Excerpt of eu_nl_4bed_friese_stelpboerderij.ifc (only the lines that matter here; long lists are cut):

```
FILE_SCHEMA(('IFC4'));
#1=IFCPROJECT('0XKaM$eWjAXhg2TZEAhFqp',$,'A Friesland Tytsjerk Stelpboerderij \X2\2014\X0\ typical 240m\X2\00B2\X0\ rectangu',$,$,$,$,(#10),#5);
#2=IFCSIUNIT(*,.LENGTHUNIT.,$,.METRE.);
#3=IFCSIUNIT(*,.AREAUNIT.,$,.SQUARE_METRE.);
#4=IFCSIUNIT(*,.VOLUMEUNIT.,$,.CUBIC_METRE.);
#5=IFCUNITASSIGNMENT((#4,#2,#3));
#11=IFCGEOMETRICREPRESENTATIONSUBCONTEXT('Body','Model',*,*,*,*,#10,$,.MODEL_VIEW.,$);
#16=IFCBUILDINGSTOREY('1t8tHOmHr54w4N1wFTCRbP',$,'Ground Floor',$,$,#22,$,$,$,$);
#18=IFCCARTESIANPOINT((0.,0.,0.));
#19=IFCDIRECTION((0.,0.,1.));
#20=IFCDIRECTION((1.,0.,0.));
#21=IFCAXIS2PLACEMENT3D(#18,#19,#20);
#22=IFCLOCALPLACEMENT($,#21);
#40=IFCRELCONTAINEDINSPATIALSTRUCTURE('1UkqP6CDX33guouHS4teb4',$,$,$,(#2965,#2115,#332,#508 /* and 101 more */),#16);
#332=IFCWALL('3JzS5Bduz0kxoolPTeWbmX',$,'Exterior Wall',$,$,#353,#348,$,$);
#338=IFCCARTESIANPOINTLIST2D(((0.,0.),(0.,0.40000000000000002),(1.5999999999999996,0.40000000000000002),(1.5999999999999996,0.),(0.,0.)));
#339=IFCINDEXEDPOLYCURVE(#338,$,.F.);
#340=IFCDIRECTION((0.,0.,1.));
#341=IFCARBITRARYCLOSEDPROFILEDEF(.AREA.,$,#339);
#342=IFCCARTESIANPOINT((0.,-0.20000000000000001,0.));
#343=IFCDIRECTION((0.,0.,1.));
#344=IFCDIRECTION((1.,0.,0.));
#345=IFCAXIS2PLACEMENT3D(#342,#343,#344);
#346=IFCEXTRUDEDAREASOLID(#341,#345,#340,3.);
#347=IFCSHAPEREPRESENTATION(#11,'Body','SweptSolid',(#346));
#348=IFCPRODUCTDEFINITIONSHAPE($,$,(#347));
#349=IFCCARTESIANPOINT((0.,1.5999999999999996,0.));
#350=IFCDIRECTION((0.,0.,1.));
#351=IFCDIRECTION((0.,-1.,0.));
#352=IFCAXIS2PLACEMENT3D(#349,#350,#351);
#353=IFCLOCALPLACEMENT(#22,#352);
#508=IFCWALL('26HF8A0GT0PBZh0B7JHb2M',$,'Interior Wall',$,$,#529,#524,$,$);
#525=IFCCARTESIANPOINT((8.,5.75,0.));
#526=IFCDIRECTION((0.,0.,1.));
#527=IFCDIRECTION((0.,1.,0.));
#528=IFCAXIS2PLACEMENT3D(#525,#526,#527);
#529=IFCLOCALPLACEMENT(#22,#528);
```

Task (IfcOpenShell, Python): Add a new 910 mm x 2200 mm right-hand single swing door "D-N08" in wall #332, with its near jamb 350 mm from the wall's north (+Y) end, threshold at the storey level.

```python
import numpy as np
import ifcopenshell
import ifcopenshell.api.feature
import ifcopenshell.api.geometry
import ifcopenshell.api.root
import ifcopenshell.api.spatial
import ifcopenshell.geom
import ifcopenshell.util.element
import ifcopenshell.util.placement
import ifcopenshell.util.representation
import ifcopenshell.util.shape
import ifcopenshell.util.unit

model = ifcopenshell.open("eu_nl_4bed_friese_stelpboerderij.ifc")
unit_scale = ifcopenshell.util.unit.calculate_unit_scale(model)
settings = ifcopenshell.geom.settings()


def volume(element):
    """Net volume in cubic metres, openings subtracted."""
    shape = ifcopenshell.geom.create_shape(settings, element)
    return ifcopenshell.util.shape.get_volume(shape.geometry)


wall = model.by_id(332)
storey = ifcopenshell.util.element.get_container(wall, ifc_class="IfcBuildingStorey")
context = ifcopenshell.util.representation.get_context(model, "Model", "Body", "MODEL_VIEW")
before = volume(wall)

width, height, from_end, sill = 0.91, 2.2, 0.35, 0.0  # metres

# The wall runs along its own X axis, and the end named is its -X end.
wall_shape = ifcopenshell.geom.create_shape(settings, wall)
x, y, z = ifcopenshell.util.shape.get_vertices(wall_shape.geometry).T
start = x.min() + from_end
face, thickness = float(y.min()), float(y.max() - y.min())
wall_matrix = ifcopenshell.util.placement.get_local_placement(wall.ObjectPlacement)
level = ifcopenshell.util.placement.get_local_placement(storey.ObjectPlacement)[2, 3]


def in_wall(x, y):
    """Placement at x, y metres in the wall's axes, at sill height."""
    matrix = wall_matrix.copy()
    matrix[:, 3] = wall_matrix @ np.array([x / unit_scale, y / unit_scale, 0.0, 1.0])
    matrix[2, 3] = level + sill / unit_scale
    return matrix


# Opening: a box that overshoots both wall faces by 50 mm.
opening = ifcopenshell.api.root.create_entity(model, ifc_class="IfcOpeningElement", predefined_type="OPENING")
box = ifcopenshell.api.geometry.add_wall_representation(
    model, context=context, length=width, height=height, thickness=thickness + 0.1
)
ifcopenshell.api.geometry.assign_representation(model, product=opening, representation=box)
ifcopenshell.api.geometry.edit_object_placement(model, product=opening, matrix=in_wall(start, face - 0.05), is_si=False)
ifcopenshell.api.feature.add_feature(model, feature=opening, element=wall)

door = ifcopenshell.api.root.create_entity(model, ifc_class="IfcDoor", name="D-N08", predefined_type="DOOR")
door.OverallWidth, door.OverallHeight = width / unit_scale, height / unit_scale
door.OperationType = "SINGLE_SWING_RIGHT"
body = ifcopenshell.api.geometry.add_door_representation(
    model,
    context=context,
    overall_width=door.OverallWidth,
    overall_height=door.OverallHeight,
    operation_type="SINGLE_SWING_RIGHT",
    lining_properties={"LiningDepth": thickness / unit_scale, "ThresholdDepth": thickness / unit_scale},
)
ifcopenshell.api.geometry.assign_representation(model, product=door, representation=body)
ifcopenshell.api.spatial.assign_container(model, products=[door], relating_structure=storey)
ifcopenshell.api.feature.add_filling(model, opening=opening, element=door)

# The lining spans the wall, so the door starts at the wall face.
ifcopenshell.api.geometry.edit_object_placement(model, product=door, matrix=in_wall(start, face), is_si=False)

after = volume(wall)

print(f"wall volume {before:.3f} -> {after:.3f} m3")

model.write("eu_nl_4bed_friese_stelpboerderij-out.ifc")
```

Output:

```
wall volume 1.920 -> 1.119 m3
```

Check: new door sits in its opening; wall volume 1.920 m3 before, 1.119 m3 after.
